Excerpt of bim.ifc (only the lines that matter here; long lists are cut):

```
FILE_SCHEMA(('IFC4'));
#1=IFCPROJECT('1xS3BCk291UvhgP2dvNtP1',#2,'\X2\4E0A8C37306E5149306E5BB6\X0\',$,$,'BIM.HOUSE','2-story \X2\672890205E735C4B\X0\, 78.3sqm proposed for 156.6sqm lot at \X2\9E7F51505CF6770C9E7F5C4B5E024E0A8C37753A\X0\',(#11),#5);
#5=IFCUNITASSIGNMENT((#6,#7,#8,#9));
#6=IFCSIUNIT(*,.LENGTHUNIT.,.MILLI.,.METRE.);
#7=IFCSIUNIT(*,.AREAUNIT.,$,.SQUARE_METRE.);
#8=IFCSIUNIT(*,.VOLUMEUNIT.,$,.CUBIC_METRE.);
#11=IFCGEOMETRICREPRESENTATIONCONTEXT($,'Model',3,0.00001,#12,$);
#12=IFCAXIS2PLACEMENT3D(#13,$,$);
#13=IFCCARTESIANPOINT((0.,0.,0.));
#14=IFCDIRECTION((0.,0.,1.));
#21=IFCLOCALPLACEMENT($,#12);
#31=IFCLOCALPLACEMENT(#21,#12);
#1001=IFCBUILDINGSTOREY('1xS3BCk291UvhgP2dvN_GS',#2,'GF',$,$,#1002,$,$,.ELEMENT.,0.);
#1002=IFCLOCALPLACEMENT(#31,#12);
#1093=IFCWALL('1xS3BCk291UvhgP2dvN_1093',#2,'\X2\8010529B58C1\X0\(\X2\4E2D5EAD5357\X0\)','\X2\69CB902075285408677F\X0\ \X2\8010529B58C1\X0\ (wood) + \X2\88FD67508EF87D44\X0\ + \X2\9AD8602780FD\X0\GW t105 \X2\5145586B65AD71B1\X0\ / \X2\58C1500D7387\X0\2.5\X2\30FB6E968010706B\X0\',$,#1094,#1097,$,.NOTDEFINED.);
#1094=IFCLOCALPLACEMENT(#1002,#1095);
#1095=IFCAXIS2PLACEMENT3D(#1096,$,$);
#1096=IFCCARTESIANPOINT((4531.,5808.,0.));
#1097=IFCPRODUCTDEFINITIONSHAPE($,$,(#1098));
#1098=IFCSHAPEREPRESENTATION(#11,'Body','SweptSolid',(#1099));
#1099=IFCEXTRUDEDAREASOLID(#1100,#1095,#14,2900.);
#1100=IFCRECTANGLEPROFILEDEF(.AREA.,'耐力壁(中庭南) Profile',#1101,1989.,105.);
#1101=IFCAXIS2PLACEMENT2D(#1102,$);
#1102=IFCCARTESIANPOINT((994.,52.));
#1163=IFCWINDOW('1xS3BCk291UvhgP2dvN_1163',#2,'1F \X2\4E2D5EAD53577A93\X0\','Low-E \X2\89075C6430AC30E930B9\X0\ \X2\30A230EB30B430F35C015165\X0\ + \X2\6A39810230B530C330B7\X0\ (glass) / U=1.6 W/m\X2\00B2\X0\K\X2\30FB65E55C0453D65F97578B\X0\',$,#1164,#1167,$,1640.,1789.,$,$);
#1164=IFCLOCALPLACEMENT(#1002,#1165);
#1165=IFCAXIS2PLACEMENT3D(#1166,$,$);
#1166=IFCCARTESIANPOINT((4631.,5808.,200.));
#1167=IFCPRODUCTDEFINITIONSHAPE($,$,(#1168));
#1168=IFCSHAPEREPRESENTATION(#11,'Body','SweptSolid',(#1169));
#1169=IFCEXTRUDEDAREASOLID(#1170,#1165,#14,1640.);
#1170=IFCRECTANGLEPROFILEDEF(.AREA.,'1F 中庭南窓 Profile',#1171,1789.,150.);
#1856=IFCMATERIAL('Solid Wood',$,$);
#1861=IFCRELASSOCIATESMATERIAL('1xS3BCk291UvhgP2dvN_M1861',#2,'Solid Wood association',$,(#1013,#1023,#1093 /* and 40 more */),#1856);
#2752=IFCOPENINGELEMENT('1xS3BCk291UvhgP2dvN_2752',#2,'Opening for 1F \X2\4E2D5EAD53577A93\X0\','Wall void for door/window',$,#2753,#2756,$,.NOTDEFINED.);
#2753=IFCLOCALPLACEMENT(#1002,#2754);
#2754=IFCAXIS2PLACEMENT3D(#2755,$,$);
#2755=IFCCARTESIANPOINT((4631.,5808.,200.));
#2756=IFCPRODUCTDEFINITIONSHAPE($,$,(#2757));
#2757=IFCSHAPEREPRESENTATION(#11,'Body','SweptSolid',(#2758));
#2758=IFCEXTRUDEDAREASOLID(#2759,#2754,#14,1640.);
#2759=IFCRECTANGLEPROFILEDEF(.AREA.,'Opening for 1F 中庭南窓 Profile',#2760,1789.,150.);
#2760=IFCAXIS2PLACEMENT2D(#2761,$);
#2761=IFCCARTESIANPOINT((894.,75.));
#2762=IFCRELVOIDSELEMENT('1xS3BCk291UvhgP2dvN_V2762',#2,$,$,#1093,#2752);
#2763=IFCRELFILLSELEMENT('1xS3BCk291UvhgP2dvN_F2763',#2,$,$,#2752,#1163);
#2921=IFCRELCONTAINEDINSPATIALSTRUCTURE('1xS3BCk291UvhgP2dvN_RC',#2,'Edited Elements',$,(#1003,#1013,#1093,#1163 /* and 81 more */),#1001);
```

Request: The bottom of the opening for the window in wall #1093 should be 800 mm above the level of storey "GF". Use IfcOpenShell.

```python
import numpy as np
import ifcopenshell
import ifcopenshell.api.geometry
import ifcopenshell.geom
import ifcopenshell.util.element
import ifcopenshell.util.placement
import ifcopenshell.util.shape
import ifcopenshell.util.unit

model = ifcopenshell.open("bim.ifc")
unit_scale = ifcopenshell.util.unit.calculate_unit_scale(model)

window = model.by_id(1163)
opening = window.FillsVoids[0].RelatingOpeningElement
storey = ifcopenshell.util.element.get_container(window, ifc_class="IfcBuildingStorey")
level = ifcopenshell.util.placement.get_local_placement(storey.ObjectPlacement)[2, 3]

# The opening's origin need not be at the sill, so measure its lowest point.
shape = ifcopenshell.geom.create_shape(ifcopenshell.geom.settings(), opening)
bottom = ifcopenshell.util.shape.get_shape_bottom_elevation(shape, shape.geometry) / unit_scale
dz = level + 0.8 / unit_scale - bottom

shift = np.array([0.0, 0.0, dz])
# The window is not placed relative to its opening, so move both.
for product in (opening, window):
    matrix = ifcopenshell.util.placement.get_local_placement(product.ObjectPlacement)
    matrix[:3, 3] += shift
    ifcopenshell.api.geometry.edit_object_placement(model, product=product, matrix=matrix, is_si=False)

print(f"moved by {dz * unit_scale:+.3f} m")

model.write("bim_edited.ifc")
```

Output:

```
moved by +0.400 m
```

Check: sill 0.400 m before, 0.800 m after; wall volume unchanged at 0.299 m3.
